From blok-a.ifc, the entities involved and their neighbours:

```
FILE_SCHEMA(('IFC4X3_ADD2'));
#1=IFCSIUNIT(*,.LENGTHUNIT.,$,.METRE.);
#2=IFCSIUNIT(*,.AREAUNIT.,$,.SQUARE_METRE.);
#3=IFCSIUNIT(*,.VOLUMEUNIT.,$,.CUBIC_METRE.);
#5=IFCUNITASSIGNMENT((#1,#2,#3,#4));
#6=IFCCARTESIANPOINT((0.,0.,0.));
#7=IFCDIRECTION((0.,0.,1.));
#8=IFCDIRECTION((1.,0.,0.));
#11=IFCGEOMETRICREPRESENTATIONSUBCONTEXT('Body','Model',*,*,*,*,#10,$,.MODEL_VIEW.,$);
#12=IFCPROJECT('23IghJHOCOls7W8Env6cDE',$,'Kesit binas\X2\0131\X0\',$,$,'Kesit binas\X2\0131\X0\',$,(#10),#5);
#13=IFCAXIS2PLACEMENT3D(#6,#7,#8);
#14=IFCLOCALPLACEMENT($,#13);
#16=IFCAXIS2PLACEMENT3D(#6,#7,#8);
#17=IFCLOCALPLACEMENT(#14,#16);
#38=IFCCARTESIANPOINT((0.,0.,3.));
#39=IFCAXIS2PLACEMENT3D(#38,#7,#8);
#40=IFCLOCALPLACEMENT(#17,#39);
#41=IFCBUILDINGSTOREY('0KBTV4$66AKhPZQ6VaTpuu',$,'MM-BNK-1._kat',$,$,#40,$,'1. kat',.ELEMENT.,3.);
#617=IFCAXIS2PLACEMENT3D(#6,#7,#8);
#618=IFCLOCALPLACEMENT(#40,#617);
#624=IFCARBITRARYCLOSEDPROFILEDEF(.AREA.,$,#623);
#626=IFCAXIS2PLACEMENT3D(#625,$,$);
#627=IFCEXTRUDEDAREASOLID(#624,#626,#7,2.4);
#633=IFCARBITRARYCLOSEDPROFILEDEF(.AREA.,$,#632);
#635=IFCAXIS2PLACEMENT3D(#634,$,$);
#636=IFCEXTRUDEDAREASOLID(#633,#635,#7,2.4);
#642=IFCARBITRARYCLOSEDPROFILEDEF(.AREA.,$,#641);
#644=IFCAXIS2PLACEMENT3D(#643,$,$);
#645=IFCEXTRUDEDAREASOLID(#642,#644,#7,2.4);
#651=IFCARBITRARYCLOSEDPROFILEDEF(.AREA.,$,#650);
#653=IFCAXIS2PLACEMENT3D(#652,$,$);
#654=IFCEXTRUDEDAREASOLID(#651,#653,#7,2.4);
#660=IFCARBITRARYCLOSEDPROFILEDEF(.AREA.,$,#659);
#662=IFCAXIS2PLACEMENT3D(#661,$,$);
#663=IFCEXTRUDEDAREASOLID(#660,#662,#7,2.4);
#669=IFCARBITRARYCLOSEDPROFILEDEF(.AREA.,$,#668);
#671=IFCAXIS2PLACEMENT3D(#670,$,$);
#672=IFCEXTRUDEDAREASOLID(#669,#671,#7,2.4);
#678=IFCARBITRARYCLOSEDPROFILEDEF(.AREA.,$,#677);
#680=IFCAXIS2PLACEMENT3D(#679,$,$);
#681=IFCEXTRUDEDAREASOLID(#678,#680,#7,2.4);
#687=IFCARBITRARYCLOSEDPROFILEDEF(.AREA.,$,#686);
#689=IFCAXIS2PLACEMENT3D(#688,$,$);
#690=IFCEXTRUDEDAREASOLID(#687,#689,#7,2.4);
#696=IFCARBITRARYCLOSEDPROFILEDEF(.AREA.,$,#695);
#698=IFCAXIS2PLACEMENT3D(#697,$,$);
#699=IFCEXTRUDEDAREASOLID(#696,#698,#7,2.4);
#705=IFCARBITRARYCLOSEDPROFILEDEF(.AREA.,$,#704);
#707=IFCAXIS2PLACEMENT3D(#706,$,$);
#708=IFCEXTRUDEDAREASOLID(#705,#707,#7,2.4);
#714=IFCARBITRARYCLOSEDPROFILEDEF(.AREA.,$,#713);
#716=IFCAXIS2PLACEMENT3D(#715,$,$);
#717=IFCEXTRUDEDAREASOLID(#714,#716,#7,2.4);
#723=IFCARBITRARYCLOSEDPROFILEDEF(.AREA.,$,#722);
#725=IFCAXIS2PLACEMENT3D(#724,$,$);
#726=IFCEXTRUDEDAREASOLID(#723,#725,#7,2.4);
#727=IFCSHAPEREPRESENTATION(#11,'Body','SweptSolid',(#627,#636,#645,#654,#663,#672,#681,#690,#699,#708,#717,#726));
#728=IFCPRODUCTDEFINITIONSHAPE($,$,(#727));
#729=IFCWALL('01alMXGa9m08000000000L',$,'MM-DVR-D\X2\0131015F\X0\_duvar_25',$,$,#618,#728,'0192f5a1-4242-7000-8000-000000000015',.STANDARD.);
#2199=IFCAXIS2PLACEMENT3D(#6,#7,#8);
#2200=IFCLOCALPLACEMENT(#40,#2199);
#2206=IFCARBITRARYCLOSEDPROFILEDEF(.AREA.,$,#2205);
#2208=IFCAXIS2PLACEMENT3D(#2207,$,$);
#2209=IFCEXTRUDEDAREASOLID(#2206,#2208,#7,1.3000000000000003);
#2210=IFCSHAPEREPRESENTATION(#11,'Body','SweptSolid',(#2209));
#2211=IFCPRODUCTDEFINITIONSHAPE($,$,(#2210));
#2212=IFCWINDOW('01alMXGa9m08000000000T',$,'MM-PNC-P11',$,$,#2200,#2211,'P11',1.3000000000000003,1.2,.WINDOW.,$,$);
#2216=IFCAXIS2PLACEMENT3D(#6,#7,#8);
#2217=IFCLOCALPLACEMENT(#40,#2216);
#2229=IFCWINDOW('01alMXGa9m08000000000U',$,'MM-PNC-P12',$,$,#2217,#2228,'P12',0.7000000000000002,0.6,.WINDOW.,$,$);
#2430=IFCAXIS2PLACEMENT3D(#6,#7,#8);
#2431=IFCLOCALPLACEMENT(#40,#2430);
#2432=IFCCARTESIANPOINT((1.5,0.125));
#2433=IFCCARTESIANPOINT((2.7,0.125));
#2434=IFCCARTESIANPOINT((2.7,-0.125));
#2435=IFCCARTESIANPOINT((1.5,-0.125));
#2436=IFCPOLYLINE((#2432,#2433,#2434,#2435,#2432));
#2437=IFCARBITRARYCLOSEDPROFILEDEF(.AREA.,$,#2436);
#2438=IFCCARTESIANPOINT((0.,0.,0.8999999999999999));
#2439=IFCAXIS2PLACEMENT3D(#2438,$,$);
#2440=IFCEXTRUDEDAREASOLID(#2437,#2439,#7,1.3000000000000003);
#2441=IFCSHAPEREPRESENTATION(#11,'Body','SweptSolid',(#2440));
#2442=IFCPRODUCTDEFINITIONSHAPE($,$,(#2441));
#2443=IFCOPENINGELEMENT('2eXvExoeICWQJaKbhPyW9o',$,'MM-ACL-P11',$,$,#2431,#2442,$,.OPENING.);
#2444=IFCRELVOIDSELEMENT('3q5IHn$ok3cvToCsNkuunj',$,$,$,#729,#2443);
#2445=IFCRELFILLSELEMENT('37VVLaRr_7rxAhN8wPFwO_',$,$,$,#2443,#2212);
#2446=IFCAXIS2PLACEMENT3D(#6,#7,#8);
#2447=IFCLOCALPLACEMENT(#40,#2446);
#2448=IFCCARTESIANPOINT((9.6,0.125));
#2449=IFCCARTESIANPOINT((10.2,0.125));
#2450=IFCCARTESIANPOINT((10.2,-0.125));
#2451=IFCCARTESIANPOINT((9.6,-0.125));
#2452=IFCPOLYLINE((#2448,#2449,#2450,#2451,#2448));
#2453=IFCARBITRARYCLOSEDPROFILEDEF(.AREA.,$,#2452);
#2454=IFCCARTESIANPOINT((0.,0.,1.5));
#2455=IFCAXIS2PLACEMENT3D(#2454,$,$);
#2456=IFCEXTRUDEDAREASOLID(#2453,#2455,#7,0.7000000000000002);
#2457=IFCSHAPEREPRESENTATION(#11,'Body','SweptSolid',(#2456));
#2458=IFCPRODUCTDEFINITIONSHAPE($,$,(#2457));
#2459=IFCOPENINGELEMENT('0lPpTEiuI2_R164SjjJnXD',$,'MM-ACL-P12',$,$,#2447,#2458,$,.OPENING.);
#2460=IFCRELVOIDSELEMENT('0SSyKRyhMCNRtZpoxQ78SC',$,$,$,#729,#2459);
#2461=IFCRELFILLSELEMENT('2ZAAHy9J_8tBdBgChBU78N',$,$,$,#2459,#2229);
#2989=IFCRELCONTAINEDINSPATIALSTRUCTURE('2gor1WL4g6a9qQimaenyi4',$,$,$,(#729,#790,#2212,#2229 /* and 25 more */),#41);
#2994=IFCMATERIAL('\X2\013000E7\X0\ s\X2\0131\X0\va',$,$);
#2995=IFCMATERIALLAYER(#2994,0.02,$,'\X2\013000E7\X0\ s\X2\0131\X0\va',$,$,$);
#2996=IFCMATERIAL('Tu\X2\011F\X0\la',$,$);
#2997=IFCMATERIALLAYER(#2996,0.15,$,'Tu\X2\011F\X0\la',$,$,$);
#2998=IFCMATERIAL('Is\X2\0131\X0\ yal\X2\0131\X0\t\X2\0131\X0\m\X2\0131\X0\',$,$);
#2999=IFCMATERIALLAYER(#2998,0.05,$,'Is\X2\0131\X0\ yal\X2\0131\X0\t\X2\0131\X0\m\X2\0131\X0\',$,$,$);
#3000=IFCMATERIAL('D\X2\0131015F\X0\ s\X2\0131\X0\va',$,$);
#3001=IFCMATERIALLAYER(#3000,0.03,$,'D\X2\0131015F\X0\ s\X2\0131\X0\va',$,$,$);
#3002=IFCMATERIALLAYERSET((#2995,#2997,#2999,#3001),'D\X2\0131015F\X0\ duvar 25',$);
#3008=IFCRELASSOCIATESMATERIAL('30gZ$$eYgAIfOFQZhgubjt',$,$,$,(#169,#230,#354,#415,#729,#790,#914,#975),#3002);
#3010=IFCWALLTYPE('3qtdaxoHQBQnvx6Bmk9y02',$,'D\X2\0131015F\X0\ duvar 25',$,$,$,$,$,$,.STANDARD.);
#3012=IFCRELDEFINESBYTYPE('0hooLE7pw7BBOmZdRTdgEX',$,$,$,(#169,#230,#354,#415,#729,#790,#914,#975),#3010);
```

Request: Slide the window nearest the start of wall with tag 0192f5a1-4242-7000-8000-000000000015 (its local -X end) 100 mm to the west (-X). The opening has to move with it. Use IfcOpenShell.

```python
import ifcopenshell
import ifcopenshell.api.geometry
import ifcopenshell.util.placement
import ifcopenshell.util.unit

model = ifcopenshell.open("blok-a.ifc")
unit_scale = ifcopenshell.util.unit.calculate_unit_scale(model)

window = model.by_guid("01alMXGa9m08000000000T")
opening = window.FillsVoids[0].RelatingOpeningElement
wall = opening.VoidsElements[0].RelatingBuildingElement

wall_matrix = ifcopenshell.util.placement.get_local_placement(wall.ObjectPlacement)
shift = wall_matrix[:3, 0] * -0.1 / unit_scale
before = ifcopenshell.util.placement.get_local_placement(window.ObjectPlacement)[:3, 3].copy()

# The window is not placed relative to its opening, so move both.
for product in (opening, window):
    matrix = ifcopenshell.util.placement.get_local_placement(product.ObjectPlacement)
    matrix[:3, 3] += shift
    ifcopenshell.api.geometry.edit_object_placement(model, product=product, matrix=matrix, is_si=False)

after = ifcopenshell.util.placement.get_local_placement(window.ObjectPlacement)[:3, 3]
print("window moved by", (after - before).round(3) + 0.0)

model.write("blok-a_v2.ifc")
```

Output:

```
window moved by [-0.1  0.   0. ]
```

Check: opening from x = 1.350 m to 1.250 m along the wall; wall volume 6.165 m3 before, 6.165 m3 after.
